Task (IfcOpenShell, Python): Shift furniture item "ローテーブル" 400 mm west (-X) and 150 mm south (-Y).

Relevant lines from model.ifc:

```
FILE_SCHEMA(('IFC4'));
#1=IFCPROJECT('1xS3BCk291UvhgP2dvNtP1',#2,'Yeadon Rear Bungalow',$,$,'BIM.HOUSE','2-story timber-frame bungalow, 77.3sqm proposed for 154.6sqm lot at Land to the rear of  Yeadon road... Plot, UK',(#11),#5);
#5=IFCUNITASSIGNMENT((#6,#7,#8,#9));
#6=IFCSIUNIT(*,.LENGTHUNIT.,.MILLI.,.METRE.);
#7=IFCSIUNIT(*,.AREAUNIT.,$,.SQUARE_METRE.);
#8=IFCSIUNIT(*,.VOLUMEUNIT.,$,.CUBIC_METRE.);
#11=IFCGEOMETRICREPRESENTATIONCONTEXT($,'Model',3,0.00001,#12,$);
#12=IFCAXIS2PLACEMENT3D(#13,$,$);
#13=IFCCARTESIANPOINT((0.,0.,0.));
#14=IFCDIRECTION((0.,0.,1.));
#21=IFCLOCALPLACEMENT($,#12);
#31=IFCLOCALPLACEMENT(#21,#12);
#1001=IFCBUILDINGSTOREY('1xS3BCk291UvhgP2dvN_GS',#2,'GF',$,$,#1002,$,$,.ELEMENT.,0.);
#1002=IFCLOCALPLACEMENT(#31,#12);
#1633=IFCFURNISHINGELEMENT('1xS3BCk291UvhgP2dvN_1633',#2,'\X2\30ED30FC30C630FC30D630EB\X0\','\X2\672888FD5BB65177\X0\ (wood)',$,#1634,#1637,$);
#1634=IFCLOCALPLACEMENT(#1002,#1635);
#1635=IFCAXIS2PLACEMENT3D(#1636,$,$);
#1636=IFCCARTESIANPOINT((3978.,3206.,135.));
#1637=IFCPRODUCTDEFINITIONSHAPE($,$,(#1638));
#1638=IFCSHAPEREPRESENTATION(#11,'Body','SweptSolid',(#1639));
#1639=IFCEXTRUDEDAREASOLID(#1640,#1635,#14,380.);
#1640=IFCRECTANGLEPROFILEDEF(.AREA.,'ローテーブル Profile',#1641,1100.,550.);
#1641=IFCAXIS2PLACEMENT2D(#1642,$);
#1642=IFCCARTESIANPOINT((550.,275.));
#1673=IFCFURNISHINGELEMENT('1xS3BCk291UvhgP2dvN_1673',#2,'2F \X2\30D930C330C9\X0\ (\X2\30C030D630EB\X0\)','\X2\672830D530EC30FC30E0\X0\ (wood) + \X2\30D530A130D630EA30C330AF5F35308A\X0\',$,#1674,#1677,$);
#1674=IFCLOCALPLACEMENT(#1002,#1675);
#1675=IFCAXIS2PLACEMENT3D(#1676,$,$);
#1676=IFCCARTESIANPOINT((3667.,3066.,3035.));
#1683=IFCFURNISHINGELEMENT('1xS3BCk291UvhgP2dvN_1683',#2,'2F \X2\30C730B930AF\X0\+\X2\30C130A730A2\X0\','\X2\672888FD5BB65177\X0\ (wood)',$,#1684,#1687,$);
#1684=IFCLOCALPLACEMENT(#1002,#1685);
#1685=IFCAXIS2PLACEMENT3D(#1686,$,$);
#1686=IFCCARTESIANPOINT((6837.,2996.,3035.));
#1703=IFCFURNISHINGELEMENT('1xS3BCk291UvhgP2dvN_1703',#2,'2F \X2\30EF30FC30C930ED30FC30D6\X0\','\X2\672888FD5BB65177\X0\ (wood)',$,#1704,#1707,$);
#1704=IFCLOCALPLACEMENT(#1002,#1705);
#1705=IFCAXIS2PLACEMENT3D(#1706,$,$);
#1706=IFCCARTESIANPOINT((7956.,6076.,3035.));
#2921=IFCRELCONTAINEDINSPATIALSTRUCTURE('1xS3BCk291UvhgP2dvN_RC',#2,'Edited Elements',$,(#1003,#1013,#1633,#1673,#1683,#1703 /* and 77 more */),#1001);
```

```python
import ifcopenshell
import ifcopenshell.api.geometry
import ifcopenshell.util.placement
import ifcopenshell.util.unit

model = ifcopenshell.open("model.ifc")
unit_scale = ifcopenshell.util.unit.calculate_unit_scale(model)

item = model.by_id(1633)
matrix = ifcopenshell.util.placement.get_local_placement(item.ObjectPlacement)
matrix[0, 3] -= 0.4 / unit_scale
matrix[1, 3] -= 0.15 / unit_scale
ifcopenshell.api.geometry.edit_object_placement(model, product=item, matrix=matrix, is_si=False)

print(ifcopenshell.util.placement.get_local_placement(item.ObjectPlacement).round(3) + 0.0)

model.write("model_rev.ifc")
```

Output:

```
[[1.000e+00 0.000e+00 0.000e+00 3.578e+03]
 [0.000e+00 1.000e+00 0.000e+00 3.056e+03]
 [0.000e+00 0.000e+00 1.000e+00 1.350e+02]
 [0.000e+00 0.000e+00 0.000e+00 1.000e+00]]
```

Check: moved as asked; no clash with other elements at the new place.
